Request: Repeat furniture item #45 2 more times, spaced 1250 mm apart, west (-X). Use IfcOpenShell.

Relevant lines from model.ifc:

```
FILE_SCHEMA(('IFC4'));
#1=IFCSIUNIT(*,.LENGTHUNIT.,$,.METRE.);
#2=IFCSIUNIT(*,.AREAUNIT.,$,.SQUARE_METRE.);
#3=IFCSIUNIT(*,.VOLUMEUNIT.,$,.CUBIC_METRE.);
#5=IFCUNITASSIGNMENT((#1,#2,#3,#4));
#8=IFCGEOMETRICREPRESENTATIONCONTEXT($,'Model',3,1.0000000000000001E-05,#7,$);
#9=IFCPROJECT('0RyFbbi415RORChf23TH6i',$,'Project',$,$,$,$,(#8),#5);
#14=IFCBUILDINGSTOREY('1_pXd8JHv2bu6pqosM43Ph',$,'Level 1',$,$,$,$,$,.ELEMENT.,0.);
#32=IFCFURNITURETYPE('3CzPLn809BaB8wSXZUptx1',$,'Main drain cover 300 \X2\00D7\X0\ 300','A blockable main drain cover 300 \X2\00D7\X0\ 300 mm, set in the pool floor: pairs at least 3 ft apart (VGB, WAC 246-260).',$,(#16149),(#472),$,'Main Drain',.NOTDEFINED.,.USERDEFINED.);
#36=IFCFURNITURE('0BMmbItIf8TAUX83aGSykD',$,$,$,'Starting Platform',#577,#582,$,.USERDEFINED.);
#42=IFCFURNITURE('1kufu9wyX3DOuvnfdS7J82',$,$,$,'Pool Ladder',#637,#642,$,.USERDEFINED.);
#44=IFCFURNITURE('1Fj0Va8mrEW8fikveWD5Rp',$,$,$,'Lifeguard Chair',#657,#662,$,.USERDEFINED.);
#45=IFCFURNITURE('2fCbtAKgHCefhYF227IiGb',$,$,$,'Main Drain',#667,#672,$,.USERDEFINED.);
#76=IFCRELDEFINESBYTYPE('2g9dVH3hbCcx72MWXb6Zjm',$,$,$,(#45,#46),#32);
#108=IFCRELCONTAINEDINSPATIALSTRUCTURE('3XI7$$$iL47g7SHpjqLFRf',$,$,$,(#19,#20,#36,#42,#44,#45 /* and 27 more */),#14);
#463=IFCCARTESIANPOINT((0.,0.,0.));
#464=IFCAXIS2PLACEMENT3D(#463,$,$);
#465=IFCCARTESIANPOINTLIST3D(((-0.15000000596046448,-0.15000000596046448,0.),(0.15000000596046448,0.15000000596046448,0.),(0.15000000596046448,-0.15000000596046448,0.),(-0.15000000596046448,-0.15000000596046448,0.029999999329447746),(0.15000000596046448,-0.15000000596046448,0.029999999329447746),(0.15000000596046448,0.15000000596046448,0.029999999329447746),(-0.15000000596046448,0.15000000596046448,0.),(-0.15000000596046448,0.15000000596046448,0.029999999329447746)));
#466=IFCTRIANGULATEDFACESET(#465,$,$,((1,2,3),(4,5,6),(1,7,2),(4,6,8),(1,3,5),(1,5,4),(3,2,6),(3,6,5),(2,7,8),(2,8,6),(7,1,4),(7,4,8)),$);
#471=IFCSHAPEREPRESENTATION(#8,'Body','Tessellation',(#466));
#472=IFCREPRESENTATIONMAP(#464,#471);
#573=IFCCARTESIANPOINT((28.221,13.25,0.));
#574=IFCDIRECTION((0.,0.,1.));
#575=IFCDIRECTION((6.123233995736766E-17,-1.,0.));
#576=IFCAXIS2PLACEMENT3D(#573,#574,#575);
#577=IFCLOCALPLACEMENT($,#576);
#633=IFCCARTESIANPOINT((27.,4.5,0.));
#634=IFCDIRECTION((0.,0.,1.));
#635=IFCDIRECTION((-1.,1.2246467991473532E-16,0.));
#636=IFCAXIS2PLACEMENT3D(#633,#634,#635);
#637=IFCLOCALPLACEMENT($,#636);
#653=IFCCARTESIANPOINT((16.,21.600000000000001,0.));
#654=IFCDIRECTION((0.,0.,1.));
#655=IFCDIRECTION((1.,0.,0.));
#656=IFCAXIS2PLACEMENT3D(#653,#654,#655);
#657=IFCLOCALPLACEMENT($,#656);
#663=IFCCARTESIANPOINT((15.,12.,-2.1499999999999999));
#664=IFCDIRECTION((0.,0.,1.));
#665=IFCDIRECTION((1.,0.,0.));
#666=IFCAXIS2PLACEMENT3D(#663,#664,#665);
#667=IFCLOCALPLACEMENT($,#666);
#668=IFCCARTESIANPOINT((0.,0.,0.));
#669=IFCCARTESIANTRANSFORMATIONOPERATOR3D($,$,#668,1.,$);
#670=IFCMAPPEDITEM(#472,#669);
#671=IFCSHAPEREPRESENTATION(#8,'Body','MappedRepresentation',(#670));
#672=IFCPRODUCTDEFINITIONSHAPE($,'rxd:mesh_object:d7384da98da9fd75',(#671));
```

```python
import numpy as np
import ifcopenshell
import ifcopenshell.api.geometry
import ifcopenshell.api.root
import ifcopenshell.util.element
import ifcopenshell.util.placement

model = ifcopenshell.open("model.ifc")

source = model.by_id(45)
base = ifcopenshell.util.placement.get_local_placement(source.ObjectPlacement)
step = np.array([-1.0, 0.0, 0.0]) * 1.25

for i in range(1, 3):
    copy = ifcopenshell.api.root.copy_class(model, product=source)
    copy.Representation = ifcopenshell.util.element.copy_deep(
        model, source.Representation, exclude=["IfcGeometricRepresentationContext", "IfcRepresentationMap"]
    )
    matrix = base.copy()
    matrix[:3, 3] += i * step
    print("added at", matrix[:3, 3].round(3) + 0.0)
    ifcopenshell.api.geometry.edit_object_placement(model, product=copy, matrix=matrix, is_si=False)

model.write("model_v2.ifc")
```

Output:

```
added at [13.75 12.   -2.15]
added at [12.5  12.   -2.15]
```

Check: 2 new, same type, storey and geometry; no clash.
